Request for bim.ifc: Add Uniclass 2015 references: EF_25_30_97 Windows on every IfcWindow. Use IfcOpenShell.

First a look at what the model holds.

```python
import ifcopenshell

model = ifcopenshell.open("bim.ifc")
print(model.schema)
print("classifications:", [c.Name for c in model.by_type("IfcClassification")])
for ifc_class in ("IfcDoor", "IfcRoof", "IfcStair", "IfcWall", "IfcWindow"):
    print(ifc_class, len(model.by_type(ifc_class)))
```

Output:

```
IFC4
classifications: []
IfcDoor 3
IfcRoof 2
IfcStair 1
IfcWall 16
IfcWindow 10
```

```python
import ifcopenshell
import ifcopenshell.api.classification

model = ifcopenshell.open("bim.ifc")

system = ifcopenshell.api.classification.add_classification(model, classification="Uniclass 2015")

codes = {
    "IfcWindow": ("EF_25_30_97", "Windows"),
}
for ifc_class, (code, name) in codes.items():
    products = model.by_type(ifc_class)
    ifcopenshell.api.classification.add_reference(
        model, products=products, classification=system, identification=code, name=name
    )
    print(code, len(products))

model.write("bim-out.ifc")
```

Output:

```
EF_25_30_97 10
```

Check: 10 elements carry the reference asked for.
